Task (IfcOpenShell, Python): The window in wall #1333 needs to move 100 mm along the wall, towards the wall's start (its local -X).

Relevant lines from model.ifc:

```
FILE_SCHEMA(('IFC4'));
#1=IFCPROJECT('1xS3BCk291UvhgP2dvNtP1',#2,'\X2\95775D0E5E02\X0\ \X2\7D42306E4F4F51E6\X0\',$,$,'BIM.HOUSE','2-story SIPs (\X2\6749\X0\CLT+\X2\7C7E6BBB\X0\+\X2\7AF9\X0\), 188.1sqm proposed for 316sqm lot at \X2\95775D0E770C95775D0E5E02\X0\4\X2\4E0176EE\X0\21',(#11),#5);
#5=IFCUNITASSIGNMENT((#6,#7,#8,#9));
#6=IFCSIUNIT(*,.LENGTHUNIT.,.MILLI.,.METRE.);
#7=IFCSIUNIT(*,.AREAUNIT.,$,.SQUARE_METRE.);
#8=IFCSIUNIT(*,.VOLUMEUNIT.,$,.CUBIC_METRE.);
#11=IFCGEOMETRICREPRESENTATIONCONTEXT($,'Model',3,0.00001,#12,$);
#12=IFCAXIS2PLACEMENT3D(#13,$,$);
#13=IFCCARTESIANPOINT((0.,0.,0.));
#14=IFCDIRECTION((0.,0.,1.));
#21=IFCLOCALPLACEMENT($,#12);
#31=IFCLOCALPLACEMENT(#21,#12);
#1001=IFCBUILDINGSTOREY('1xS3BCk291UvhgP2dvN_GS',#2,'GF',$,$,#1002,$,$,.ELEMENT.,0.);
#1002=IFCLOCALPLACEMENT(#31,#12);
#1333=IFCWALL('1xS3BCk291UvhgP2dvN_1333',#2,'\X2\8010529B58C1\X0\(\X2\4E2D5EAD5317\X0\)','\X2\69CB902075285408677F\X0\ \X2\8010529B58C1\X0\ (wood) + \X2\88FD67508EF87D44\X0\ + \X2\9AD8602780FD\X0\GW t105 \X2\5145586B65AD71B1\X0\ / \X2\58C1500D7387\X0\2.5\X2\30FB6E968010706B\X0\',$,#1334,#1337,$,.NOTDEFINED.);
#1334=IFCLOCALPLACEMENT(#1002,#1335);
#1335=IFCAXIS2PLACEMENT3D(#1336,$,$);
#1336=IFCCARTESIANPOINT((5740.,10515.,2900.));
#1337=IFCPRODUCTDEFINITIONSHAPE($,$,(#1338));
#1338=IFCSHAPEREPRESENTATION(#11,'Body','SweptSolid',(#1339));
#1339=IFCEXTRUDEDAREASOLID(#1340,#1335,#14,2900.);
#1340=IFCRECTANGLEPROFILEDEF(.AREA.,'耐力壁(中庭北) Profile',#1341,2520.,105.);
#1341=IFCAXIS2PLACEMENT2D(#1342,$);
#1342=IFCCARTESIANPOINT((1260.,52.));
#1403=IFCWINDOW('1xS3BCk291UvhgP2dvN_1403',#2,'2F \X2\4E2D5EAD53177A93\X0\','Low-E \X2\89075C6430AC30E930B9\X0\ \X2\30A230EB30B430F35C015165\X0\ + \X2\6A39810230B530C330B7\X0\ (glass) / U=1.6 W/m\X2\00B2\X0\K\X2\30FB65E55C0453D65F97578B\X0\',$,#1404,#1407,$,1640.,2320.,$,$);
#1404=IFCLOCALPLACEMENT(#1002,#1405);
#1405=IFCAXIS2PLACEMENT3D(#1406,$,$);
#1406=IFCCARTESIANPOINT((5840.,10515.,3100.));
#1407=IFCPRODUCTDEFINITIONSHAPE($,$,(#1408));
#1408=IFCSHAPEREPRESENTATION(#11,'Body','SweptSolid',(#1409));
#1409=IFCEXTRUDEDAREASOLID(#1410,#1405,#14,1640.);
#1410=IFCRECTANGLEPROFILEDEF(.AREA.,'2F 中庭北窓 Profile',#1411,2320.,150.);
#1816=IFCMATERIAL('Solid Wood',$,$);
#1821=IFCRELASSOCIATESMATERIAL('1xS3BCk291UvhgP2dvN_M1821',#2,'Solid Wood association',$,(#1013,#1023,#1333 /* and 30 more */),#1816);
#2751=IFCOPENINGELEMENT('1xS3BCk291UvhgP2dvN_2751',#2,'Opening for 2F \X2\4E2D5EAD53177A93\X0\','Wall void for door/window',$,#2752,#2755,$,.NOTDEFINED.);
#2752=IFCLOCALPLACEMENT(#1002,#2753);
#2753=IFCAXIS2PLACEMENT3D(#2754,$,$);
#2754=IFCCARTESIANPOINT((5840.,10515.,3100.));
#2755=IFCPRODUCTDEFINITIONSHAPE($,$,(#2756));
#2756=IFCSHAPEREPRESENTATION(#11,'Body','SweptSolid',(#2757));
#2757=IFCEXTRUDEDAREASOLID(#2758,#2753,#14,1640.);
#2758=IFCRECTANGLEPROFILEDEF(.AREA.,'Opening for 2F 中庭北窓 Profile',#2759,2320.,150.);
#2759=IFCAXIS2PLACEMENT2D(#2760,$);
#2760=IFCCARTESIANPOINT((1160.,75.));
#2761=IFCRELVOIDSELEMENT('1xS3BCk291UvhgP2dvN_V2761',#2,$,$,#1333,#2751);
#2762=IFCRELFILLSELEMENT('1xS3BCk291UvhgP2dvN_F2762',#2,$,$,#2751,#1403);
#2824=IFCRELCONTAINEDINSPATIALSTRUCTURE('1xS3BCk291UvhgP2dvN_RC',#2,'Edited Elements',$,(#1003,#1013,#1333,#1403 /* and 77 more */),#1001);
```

```python
import ifcopenshell
import ifcopenshell.api.geometry
import ifcopenshell.util.placement
import ifcopenshell.util.unit

model = ifcopenshell.open("model.ifc")
unit_scale = ifcopenshell.util.unit.calculate_unit_scale(model)

window = model.by_id(1403)
opening = window.FillsVoids[0].RelatingOpeningElement
wall = opening.VoidsElements[0].RelatingBuildingElement

wall_matrix = ifcopenshell.util.placement.get_local_placement(wall.ObjectPlacement)
shift = wall_matrix[:3, 0] * -0.1 / unit_scale
before = ifcopenshell.util.placement.get_local_placement(window.ObjectPlacement)[:3, 3].copy()

# The window is not placed relative to its opening, so move both.
for product in (opening, window):
    matrix = ifcopenshell.util.placement.get_local_placement(product.ObjectPlacement)
    matrix[:3, 3] += shift
    ifcopenshell.api.geometry.edit_object_placement(model, product=product, matrix=matrix, is_si=False)

after = ifcopenshell.util.placement.get_local_placement(window.ObjectPlacement)[:3, 3]
print("window moved by", (after - before).round(3) + 0.0)

model.write("model_updated.ifc")
```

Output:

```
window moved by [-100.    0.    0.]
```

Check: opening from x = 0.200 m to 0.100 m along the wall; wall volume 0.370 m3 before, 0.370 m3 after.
